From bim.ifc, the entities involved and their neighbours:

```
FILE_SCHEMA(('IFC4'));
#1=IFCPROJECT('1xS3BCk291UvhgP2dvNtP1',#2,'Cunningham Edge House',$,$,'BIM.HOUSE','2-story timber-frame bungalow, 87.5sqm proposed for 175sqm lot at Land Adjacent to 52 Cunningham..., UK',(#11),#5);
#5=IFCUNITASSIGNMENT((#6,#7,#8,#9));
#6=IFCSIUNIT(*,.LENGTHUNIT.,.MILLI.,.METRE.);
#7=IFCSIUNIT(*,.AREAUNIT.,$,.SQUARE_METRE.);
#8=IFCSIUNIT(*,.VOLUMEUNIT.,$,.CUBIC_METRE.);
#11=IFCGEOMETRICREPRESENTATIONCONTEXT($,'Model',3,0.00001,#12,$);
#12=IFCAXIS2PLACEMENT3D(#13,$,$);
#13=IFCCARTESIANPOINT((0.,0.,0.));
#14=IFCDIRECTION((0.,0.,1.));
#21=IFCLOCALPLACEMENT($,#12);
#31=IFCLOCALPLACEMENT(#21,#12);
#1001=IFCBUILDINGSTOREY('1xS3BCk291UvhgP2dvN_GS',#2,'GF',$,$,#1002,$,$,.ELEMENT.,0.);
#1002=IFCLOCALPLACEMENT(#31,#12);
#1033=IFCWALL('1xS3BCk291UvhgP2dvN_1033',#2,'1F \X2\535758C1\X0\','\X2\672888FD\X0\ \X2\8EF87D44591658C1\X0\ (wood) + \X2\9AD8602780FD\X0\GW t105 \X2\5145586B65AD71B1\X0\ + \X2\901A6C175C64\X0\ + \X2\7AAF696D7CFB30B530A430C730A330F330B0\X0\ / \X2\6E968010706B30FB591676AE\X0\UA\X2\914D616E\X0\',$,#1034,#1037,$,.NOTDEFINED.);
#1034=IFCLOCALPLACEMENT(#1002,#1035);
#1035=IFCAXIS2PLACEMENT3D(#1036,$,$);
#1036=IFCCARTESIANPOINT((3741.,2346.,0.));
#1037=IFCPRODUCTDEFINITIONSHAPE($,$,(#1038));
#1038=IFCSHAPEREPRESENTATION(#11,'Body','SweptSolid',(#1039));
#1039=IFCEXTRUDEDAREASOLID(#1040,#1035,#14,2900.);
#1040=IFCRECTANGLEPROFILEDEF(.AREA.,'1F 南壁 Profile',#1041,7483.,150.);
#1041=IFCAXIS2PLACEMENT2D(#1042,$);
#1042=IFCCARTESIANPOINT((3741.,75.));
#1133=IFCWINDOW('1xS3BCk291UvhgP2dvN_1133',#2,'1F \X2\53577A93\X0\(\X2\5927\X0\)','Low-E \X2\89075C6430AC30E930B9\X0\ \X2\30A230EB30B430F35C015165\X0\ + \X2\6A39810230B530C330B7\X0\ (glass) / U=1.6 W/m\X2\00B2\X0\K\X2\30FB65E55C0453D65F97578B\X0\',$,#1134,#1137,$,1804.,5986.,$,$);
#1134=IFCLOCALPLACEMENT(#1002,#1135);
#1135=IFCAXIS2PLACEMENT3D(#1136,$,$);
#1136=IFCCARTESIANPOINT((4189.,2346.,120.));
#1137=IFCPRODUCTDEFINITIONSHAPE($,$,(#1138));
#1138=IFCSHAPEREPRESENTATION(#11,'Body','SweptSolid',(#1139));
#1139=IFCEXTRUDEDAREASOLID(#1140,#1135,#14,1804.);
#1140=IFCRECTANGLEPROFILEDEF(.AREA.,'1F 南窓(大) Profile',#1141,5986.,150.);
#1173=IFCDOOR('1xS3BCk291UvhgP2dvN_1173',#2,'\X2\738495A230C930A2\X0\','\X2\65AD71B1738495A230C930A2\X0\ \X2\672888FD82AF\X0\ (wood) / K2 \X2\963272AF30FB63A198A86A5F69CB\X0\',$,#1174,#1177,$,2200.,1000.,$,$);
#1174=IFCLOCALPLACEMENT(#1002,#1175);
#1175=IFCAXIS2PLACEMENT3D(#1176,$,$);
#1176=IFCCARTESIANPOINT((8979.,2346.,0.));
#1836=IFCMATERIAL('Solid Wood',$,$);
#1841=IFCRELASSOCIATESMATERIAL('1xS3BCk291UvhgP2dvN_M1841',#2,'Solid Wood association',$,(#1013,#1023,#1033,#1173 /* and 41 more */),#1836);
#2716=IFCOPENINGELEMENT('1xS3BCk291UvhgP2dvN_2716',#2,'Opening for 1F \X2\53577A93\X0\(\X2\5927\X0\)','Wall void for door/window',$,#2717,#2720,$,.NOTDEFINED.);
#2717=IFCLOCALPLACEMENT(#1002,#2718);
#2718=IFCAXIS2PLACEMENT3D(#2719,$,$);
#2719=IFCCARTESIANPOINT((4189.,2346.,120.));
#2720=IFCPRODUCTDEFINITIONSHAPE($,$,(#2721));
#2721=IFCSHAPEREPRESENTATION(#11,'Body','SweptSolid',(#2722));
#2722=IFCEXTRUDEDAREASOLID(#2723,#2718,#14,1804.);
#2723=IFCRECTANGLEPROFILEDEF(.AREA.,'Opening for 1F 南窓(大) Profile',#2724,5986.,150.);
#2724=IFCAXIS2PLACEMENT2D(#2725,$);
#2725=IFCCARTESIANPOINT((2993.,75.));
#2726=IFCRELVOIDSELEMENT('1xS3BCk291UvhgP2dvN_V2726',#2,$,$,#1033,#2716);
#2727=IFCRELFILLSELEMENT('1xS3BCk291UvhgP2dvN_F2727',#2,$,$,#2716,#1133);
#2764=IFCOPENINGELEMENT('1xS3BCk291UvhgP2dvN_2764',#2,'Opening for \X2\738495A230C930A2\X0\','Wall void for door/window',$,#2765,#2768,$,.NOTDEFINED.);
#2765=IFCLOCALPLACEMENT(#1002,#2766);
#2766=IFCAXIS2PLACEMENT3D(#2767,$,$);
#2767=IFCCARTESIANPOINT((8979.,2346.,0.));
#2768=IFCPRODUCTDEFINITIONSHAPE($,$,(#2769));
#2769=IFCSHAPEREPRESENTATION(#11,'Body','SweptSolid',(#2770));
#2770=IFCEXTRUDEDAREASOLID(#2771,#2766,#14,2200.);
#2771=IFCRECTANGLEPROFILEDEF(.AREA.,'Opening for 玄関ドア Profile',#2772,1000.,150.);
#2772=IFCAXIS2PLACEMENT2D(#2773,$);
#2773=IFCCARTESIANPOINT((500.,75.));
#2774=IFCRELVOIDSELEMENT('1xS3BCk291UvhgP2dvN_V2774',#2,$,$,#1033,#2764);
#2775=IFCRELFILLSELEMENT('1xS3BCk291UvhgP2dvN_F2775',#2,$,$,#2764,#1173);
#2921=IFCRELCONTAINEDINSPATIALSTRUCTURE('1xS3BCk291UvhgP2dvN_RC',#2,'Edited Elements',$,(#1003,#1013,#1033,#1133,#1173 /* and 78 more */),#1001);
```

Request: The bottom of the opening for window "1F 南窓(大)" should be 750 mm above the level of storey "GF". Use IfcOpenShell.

```python
import numpy as np
import ifcopenshell
import ifcopenshell.api.geometry
import ifcopenshell.geom
import ifcopenshell.util.element
import ifcopenshell.util.placement
import ifcopenshell.util.shape
import ifcopenshell.util.unit

model = ifcopenshell.open("bim.ifc")
unit_scale = ifcopenshell.util.unit.calculate_unit_scale(model)

window = model.by_guid("1xS3BCk291UvhgP2dvN_1133")
opening = window.FillsVoids[0].RelatingOpeningElement
storey = ifcopenshell.util.element.get_container(window, ifc_class="IfcBuildingStorey")
level = ifcopenshell.util.placement.get_local_placement(storey.ObjectPlacement)[2, 3]

# The opening's origin need not be at the sill, so measure its lowest point.
shape = ifcopenshell.geom.create_shape(ifcopenshell.geom.settings(), opening)
bottom = ifcopenshell.util.shape.get_shape_bottom_elevation(shape, shape.geometry) / unit_scale
dz = level + 750.0 - bottom

shift = np.array([0.0, 0.0, dz])
# The window is not placed relative to its opening, so move both.
for product in (opening, window):
    matrix = ifcopenshell.util.placement.get_local_placement(product.ObjectPlacement)
    matrix[:3, 3] += shift
    ifcopenshell.api.geometry.edit_object_placement(model, product=product, matrix=matrix, is_si=False)

print(f"moved by {dz * unit_scale:+.3f} m")

model.write("bim_edited.ifc")
```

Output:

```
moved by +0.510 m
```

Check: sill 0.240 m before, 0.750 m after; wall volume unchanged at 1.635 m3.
